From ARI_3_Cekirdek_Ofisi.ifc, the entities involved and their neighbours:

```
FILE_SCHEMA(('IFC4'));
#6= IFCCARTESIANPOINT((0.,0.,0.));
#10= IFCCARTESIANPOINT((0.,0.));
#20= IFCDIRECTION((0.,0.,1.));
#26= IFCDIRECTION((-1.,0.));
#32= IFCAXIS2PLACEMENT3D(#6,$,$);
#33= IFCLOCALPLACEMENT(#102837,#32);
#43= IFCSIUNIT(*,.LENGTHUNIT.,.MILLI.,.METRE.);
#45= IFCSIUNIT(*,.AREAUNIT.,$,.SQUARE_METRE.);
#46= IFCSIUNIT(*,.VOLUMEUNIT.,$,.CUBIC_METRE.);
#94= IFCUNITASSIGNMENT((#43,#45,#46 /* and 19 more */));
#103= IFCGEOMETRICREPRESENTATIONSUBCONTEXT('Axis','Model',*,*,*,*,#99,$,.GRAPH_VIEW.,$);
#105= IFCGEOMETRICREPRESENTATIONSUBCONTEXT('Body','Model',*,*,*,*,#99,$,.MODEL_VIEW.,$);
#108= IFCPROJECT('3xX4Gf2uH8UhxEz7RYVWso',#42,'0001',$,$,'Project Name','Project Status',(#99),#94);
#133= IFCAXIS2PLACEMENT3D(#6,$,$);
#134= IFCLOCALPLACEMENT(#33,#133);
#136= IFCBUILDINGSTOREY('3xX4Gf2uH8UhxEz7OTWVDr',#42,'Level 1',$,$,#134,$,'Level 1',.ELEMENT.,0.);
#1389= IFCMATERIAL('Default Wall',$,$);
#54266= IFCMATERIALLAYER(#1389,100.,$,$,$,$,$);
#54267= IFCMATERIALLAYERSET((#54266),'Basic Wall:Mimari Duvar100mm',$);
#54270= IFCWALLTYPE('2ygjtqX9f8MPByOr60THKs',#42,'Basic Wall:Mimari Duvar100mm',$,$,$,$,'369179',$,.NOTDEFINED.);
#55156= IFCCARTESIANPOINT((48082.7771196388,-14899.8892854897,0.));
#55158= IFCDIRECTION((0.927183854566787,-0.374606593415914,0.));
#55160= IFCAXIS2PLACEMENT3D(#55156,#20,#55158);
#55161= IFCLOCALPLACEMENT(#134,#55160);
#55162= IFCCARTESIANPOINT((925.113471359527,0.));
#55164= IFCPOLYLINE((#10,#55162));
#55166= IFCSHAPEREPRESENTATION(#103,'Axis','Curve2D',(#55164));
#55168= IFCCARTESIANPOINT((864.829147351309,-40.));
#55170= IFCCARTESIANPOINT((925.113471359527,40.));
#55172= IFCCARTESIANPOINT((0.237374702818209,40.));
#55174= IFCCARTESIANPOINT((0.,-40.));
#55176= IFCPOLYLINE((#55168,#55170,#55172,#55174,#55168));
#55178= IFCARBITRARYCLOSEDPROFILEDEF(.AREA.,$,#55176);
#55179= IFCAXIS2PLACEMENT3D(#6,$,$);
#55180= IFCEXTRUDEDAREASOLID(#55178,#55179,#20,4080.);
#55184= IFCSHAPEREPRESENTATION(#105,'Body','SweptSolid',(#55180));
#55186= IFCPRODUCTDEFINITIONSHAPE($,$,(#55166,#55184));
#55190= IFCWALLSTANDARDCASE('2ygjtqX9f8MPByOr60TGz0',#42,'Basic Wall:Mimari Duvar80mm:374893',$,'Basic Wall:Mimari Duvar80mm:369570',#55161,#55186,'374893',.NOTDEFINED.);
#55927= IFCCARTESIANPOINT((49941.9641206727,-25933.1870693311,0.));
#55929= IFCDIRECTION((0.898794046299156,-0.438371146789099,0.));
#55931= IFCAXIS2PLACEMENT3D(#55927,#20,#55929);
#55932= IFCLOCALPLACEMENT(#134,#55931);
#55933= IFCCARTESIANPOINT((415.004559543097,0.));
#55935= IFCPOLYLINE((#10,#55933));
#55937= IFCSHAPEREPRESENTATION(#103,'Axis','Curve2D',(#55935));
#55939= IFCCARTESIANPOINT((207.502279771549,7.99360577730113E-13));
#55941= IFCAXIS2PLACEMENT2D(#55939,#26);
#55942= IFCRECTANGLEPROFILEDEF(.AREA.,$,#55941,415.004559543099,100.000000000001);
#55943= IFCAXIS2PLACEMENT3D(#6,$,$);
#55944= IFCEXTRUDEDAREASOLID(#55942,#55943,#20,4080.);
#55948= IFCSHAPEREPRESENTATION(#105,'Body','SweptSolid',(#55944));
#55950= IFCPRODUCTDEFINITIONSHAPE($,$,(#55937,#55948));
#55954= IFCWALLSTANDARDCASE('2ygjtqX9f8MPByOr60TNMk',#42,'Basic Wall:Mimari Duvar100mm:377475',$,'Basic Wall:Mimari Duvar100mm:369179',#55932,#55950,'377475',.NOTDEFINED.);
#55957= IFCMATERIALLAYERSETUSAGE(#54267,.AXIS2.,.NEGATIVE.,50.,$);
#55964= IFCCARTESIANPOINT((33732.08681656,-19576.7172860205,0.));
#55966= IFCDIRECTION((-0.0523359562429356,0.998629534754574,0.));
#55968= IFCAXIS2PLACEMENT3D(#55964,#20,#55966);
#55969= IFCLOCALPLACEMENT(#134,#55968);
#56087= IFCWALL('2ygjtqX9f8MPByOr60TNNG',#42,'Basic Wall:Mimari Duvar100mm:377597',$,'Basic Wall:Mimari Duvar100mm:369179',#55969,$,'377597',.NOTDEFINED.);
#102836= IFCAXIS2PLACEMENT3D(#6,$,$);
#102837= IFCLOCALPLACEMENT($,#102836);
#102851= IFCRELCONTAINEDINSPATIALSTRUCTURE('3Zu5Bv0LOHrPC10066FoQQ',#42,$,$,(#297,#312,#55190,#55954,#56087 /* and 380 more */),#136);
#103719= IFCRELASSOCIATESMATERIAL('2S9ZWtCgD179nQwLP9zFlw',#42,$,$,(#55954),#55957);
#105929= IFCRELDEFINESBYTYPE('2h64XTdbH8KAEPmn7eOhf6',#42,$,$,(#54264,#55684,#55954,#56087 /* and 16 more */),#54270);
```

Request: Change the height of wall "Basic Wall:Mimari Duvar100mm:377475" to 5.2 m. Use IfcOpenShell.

```python
import ifcopenshell
import ifcopenshell.geom
import ifcopenshell.util.representation
import ifcopenshell.util.shape
import ifcopenshell.util.unit

model = ifcopenshell.open("ARI_3_Cekirdek_Ofisi.ifc")
unit_scale = ifcopenshell.util.unit.calculate_unit_scale(model)
settings = ifcopenshell.geom.settings()


def volume(element):
    """Net volume in cubic metres, openings subtracted."""
    shape = ifcopenshell.geom.create_shape(settings, element)
    return ifcopenshell.util.shape.get_volume(shape.geometry)


wall = model.by_guid("2ygjtqX9f8MPByOr60TNMk")
before = volume(wall)

body = ifcopenshell.util.representation.get_representation(wall, "Model", "Body")
solid = body.Items[0]
old_height = solid.Depth
solid.Depth = 5.2 / unit_scale
after = volume(wall)

print(f"height {old_height:g} -> {solid.Depth:g}, volume {before:.3f} -> {after:.3f} m3")

model.write("ARI_3_Cekirdek_Ofisi-out.ifc")
```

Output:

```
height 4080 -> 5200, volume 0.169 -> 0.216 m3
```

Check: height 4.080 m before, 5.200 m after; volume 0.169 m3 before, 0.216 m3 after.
